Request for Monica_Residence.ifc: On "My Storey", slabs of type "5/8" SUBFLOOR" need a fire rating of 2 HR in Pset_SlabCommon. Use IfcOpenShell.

First a look at what the model holds.

```python
import ifcopenshell
import ifcopenshell.util.element

model = ifcopenshell.open("Monica_Residence.ifc")
print(model.schema)
storey = next(s for s in model.by_type("IfcBuildingStorey") if s.Name == "My Storey")
slabs = [e for e in ifcopenshell.util.element.get_decomposition(storey) if e.is_a("IfcSlab")]
seen = {}
for e in slabs:
    element_type = ifcopenshell.util.element.get_type(e)
    key = (element_type.Name if element_type != e and element_type else None, ifcopenshell.util.element.get_pset(e, "Pset_SlabCommon", "FireRating"))
    seen[key] = seen.get(key, 0) + 1
for (name, value), count in sorted(seen.items(), key=str):
    print(count, "x", name, "|", value)
```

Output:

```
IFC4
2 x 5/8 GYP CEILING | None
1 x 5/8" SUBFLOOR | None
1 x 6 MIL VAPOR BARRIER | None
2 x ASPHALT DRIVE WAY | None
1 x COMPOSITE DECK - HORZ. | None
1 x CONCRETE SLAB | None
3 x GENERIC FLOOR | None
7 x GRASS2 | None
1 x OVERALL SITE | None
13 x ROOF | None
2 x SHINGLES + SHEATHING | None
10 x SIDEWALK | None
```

```python
import ifcopenshell
import ifcopenshell.api.pset
import ifcopenshell.util.element

model = ifcopenshell.open("Monica_Residence.ifc")

storey = next(s for s in model.by_type("IfcBuildingStorey") if s.Name == "My Storey")
slabs = [e for e in ifcopenshell.util.element.get_decomposition(storey) if e.is_a("IfcSlab")]

count = 0
for e in slabs:
    element_type = ifcopenshell.util.element.get_type(e)
    if element_type in (None, e) or element_type.Name != '5/8" SUBFLOOR':
        continue
    # add_pset returns the element's existing set when there is one.
    pset = ifcopenshell.api.pset.add_pset(model, product=e, name="Pset_SlabCommon")
    ifcopenshell.api.pset.edit_pset(model, pset=pset, properties={"FireRating": "2 HR"})
    count += 1

print(count, "slabs updated")

model.write("Monica_Residence_edited.ifc")
```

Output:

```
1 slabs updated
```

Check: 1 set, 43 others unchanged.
